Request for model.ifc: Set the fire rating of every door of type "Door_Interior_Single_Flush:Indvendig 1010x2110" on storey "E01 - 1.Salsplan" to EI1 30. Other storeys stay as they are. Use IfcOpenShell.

First a look at what the model holds.

```python
import ifcopenshell
import ifcopenshell.util.element

model = ifcopenshell.open("model.ifc")
print(model.schema)
storey = next(s for s in model.by_type("IfcBuildingStorey") if s.Name == "E01 - 1.Salsplan")
doors = [e for e in ifcopenshell.util.element.get_decomposition(storey) if e.is_a("IfcDoor")]
seen = {}
for e in doors:
    element_type = ifcopenshell.util.element.get_type(e)
    key = (element_type.Name if element_type != e and element_type else None, ifcopenshell.util.element.get_pset(e, "Pset_DoorCommon", "FireRating"))
    seen[key] = seen.get(key, 0) + 1
for (name, value), count in sorted(seen.items(), key=str):
    print(count, "x", name, "|", value)
```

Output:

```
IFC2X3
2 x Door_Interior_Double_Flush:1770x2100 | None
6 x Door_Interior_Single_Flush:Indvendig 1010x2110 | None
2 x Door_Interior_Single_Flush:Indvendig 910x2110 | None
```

```python
import ifcopenshell
import ifcopenshell.api.pset
import ifcopenshell.util.element

model = ifcopenshell.open("model.ifc")

storey = next(s for s in model.by_type("IfcBuildingStorey") if s.Name == "E01 - 1.Salsplan")
doors = [e for e in ifcopenshell.util.element.get_decomposition(storey) if e.is_a("IfcDoor")]

count = 0
for e in doors:
    element_type = ifcopenshell.util.element.get_type(e)
    if element_type in (None, e) or element_type.Name != "Door_Interior_Single_Flush:Indvendig 1010x2110":
        continue
    # add_pset returns the element's existing set when there is one.
    pset = ifcopenshell.api.pset.add_pset(model, product=e, name="Pset_DoorCommon")
    ifcopenshell.api.pset.edit_pset(model, pset=pset, properties={"FireRating": "EI1 30"})
    count += 1

print(count, "doors updated")

model.write("model_v2.ifc")
```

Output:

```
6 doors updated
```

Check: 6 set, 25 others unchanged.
